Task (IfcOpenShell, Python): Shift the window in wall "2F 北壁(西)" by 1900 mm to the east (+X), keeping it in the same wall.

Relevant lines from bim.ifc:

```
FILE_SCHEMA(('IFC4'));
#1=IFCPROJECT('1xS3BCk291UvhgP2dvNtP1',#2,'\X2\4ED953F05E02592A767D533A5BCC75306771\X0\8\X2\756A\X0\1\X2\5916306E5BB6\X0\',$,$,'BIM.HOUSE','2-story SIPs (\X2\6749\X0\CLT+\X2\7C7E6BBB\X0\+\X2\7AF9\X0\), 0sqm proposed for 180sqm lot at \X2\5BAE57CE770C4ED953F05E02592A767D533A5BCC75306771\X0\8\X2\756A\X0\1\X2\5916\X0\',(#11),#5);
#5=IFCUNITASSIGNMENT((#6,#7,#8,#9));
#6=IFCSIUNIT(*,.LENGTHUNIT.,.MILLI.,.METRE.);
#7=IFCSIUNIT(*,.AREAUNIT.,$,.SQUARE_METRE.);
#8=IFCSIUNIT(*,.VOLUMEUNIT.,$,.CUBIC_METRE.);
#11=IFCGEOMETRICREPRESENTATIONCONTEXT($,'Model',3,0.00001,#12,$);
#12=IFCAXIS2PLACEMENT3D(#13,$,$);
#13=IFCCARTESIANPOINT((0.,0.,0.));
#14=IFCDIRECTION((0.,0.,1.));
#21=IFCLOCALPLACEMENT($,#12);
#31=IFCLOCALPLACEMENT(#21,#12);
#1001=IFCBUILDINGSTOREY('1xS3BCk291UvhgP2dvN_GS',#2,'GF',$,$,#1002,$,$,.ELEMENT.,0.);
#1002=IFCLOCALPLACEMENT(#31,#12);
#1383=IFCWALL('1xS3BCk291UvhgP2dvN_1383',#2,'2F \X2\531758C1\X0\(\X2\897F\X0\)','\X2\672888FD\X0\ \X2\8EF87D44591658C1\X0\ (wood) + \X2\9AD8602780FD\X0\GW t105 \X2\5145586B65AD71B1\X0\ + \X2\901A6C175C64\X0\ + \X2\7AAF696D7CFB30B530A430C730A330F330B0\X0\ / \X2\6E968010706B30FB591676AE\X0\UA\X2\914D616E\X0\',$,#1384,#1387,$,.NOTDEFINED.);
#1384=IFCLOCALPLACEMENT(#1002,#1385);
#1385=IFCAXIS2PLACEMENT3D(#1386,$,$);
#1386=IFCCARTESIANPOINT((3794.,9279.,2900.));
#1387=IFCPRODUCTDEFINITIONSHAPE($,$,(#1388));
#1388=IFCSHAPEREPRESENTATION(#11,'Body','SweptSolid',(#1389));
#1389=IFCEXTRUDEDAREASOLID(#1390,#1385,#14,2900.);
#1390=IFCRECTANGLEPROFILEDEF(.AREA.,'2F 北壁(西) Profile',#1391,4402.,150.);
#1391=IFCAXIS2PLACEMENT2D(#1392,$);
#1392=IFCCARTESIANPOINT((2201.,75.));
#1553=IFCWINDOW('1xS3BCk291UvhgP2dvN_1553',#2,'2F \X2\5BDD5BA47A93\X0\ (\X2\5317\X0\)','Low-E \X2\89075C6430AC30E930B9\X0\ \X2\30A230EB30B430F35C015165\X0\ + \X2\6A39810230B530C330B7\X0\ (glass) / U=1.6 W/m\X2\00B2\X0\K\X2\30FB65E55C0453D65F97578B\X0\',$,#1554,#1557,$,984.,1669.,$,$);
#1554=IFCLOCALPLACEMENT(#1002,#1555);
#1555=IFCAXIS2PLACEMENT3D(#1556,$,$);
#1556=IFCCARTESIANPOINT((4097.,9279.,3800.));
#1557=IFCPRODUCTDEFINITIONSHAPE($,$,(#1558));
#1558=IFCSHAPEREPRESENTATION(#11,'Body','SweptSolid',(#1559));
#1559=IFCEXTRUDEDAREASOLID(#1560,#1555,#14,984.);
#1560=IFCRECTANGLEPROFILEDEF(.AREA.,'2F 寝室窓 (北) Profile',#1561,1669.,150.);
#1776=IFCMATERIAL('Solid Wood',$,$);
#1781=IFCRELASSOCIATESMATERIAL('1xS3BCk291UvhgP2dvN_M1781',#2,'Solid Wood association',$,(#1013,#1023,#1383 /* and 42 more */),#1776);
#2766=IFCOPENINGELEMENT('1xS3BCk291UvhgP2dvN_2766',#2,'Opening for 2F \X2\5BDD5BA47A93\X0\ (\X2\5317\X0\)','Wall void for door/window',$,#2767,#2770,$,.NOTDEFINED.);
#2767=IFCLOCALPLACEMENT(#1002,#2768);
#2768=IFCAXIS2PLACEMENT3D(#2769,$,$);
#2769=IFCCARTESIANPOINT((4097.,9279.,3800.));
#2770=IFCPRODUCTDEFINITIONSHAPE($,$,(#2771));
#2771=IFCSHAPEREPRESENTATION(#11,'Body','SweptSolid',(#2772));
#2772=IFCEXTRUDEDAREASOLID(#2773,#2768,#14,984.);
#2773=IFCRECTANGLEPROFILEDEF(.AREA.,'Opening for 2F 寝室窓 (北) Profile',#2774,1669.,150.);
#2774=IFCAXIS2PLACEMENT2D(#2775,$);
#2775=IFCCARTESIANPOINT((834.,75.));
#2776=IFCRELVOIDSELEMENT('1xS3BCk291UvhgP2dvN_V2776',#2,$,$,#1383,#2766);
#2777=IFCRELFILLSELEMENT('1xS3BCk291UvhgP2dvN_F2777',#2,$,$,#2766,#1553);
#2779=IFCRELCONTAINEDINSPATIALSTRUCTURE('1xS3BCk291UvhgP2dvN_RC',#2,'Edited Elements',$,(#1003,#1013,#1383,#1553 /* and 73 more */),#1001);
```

```python
import ifcopenshell
import ifcopenshell.api.geometry
import ifcopenshell.util.placement
import ifcopenshell.util.unit

model = ifcopenshell.open("bim.ifc")
unit_scale = ifcopenshell.util.unit.calculate_unit_scale(model)

window = model.by_guid("1xS3BCk291UvhgP2dvN_1553")
opening = window.FillsVoids[0].RelatingOpeningElement
wall = opening.VoidsElements[0].RelatingBuildingElement

wall_matrix = ifcopenshell.util.placement.get_local_placement(wall.ObjectPlacement)
shift = wall_matrix[:3, 0] * 1.9 / unit_scale
before = ifcopenshell.util.placement.get_local_placement(window.ObjectPlacement)[:3, 3].copy()

# The window is not placed relative to its opening, so move both.
for product in (opening, window):
    matrix = ifcopenshell.util.placement.get_local_placement(product.ObjectPlacement)
    matrix[:3, 3] += shift
    ifcopenshell.api.geometry.edit_object_placement(model, product=product, matrix=matrix, is_si=False)

after = ifcopenshell.util.placement.get_local_placement(window.ObjectPlacement)[:3, 3]
print("window moved by", (after - before).round(3) + 0.0)

model.write("bim_v2.ifc")
```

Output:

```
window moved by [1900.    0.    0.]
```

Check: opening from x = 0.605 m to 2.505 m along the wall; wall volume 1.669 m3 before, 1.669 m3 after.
